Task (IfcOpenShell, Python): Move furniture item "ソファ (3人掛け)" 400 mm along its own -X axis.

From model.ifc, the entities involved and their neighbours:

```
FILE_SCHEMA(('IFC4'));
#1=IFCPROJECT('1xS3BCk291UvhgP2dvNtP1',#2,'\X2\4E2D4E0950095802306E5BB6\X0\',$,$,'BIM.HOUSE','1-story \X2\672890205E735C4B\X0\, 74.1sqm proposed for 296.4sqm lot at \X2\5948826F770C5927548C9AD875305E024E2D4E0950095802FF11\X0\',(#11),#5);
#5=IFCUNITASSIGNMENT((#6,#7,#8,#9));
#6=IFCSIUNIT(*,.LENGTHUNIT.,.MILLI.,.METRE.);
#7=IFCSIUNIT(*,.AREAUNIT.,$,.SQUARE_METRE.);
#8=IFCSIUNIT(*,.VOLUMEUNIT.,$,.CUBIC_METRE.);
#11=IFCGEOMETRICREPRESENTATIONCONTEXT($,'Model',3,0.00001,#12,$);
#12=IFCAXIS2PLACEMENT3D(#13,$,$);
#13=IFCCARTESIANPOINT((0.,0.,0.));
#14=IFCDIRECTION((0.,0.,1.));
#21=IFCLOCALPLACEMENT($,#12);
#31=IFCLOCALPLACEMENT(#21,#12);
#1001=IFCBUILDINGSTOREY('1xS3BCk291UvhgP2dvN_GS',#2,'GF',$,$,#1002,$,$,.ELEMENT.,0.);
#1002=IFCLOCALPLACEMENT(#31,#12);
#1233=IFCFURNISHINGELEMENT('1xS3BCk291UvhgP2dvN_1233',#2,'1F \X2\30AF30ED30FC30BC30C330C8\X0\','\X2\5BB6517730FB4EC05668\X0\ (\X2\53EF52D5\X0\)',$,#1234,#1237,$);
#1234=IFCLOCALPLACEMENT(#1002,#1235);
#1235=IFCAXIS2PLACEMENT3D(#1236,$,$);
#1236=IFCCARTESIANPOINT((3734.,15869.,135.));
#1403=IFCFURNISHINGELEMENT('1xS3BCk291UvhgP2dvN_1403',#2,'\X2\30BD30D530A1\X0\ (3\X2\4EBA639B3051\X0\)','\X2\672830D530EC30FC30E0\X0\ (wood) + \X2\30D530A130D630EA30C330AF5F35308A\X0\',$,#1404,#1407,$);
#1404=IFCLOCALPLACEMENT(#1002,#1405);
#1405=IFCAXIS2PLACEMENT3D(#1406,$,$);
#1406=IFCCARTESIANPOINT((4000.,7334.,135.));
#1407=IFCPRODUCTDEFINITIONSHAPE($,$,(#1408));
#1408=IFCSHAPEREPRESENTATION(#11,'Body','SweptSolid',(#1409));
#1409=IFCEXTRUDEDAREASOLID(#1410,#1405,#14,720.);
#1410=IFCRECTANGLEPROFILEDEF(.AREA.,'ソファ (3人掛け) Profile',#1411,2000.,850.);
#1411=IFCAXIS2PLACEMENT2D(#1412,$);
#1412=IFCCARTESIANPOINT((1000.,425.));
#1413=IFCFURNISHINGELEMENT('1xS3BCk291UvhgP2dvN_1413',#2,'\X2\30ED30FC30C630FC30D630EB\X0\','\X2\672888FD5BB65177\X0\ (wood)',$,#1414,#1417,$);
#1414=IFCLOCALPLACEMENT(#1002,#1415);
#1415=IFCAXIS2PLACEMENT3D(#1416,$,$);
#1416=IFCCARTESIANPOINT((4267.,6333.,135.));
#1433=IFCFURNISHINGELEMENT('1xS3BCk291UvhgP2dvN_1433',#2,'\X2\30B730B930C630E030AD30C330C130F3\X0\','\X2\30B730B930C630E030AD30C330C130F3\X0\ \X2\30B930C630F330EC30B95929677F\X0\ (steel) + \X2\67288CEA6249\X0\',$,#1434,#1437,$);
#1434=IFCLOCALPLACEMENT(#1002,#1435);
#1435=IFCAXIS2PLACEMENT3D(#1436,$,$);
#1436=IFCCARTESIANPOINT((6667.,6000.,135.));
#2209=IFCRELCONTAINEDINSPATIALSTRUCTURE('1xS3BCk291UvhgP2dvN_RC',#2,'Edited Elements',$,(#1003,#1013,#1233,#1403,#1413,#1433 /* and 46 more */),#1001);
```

```python
import ifcopenshell
import ifcopenshell.api.geometry
import ifcopenshell.util.placement

model = ifcopenshell.open("model.ifc")

item = model.by_id(1403)
matrix = ifcopenshell.util.placement.get_local_placement(item.ObjectPlacement)
matrix[:3, 3] -= matrix[:3, 0] * 400.0
ifcopenshell.api.geometry.edit_object_placement(model, product=item, matrix=matrix, is_si=False)

print(ifcopenshell.util.placement.get_local_placement(item.ObjectPlacement).round(3) + 0.0)

model.write("model-out.ifc")
```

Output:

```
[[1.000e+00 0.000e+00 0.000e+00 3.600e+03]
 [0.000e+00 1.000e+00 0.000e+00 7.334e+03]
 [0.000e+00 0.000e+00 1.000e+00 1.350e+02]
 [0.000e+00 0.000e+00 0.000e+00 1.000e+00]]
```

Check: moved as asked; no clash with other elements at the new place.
